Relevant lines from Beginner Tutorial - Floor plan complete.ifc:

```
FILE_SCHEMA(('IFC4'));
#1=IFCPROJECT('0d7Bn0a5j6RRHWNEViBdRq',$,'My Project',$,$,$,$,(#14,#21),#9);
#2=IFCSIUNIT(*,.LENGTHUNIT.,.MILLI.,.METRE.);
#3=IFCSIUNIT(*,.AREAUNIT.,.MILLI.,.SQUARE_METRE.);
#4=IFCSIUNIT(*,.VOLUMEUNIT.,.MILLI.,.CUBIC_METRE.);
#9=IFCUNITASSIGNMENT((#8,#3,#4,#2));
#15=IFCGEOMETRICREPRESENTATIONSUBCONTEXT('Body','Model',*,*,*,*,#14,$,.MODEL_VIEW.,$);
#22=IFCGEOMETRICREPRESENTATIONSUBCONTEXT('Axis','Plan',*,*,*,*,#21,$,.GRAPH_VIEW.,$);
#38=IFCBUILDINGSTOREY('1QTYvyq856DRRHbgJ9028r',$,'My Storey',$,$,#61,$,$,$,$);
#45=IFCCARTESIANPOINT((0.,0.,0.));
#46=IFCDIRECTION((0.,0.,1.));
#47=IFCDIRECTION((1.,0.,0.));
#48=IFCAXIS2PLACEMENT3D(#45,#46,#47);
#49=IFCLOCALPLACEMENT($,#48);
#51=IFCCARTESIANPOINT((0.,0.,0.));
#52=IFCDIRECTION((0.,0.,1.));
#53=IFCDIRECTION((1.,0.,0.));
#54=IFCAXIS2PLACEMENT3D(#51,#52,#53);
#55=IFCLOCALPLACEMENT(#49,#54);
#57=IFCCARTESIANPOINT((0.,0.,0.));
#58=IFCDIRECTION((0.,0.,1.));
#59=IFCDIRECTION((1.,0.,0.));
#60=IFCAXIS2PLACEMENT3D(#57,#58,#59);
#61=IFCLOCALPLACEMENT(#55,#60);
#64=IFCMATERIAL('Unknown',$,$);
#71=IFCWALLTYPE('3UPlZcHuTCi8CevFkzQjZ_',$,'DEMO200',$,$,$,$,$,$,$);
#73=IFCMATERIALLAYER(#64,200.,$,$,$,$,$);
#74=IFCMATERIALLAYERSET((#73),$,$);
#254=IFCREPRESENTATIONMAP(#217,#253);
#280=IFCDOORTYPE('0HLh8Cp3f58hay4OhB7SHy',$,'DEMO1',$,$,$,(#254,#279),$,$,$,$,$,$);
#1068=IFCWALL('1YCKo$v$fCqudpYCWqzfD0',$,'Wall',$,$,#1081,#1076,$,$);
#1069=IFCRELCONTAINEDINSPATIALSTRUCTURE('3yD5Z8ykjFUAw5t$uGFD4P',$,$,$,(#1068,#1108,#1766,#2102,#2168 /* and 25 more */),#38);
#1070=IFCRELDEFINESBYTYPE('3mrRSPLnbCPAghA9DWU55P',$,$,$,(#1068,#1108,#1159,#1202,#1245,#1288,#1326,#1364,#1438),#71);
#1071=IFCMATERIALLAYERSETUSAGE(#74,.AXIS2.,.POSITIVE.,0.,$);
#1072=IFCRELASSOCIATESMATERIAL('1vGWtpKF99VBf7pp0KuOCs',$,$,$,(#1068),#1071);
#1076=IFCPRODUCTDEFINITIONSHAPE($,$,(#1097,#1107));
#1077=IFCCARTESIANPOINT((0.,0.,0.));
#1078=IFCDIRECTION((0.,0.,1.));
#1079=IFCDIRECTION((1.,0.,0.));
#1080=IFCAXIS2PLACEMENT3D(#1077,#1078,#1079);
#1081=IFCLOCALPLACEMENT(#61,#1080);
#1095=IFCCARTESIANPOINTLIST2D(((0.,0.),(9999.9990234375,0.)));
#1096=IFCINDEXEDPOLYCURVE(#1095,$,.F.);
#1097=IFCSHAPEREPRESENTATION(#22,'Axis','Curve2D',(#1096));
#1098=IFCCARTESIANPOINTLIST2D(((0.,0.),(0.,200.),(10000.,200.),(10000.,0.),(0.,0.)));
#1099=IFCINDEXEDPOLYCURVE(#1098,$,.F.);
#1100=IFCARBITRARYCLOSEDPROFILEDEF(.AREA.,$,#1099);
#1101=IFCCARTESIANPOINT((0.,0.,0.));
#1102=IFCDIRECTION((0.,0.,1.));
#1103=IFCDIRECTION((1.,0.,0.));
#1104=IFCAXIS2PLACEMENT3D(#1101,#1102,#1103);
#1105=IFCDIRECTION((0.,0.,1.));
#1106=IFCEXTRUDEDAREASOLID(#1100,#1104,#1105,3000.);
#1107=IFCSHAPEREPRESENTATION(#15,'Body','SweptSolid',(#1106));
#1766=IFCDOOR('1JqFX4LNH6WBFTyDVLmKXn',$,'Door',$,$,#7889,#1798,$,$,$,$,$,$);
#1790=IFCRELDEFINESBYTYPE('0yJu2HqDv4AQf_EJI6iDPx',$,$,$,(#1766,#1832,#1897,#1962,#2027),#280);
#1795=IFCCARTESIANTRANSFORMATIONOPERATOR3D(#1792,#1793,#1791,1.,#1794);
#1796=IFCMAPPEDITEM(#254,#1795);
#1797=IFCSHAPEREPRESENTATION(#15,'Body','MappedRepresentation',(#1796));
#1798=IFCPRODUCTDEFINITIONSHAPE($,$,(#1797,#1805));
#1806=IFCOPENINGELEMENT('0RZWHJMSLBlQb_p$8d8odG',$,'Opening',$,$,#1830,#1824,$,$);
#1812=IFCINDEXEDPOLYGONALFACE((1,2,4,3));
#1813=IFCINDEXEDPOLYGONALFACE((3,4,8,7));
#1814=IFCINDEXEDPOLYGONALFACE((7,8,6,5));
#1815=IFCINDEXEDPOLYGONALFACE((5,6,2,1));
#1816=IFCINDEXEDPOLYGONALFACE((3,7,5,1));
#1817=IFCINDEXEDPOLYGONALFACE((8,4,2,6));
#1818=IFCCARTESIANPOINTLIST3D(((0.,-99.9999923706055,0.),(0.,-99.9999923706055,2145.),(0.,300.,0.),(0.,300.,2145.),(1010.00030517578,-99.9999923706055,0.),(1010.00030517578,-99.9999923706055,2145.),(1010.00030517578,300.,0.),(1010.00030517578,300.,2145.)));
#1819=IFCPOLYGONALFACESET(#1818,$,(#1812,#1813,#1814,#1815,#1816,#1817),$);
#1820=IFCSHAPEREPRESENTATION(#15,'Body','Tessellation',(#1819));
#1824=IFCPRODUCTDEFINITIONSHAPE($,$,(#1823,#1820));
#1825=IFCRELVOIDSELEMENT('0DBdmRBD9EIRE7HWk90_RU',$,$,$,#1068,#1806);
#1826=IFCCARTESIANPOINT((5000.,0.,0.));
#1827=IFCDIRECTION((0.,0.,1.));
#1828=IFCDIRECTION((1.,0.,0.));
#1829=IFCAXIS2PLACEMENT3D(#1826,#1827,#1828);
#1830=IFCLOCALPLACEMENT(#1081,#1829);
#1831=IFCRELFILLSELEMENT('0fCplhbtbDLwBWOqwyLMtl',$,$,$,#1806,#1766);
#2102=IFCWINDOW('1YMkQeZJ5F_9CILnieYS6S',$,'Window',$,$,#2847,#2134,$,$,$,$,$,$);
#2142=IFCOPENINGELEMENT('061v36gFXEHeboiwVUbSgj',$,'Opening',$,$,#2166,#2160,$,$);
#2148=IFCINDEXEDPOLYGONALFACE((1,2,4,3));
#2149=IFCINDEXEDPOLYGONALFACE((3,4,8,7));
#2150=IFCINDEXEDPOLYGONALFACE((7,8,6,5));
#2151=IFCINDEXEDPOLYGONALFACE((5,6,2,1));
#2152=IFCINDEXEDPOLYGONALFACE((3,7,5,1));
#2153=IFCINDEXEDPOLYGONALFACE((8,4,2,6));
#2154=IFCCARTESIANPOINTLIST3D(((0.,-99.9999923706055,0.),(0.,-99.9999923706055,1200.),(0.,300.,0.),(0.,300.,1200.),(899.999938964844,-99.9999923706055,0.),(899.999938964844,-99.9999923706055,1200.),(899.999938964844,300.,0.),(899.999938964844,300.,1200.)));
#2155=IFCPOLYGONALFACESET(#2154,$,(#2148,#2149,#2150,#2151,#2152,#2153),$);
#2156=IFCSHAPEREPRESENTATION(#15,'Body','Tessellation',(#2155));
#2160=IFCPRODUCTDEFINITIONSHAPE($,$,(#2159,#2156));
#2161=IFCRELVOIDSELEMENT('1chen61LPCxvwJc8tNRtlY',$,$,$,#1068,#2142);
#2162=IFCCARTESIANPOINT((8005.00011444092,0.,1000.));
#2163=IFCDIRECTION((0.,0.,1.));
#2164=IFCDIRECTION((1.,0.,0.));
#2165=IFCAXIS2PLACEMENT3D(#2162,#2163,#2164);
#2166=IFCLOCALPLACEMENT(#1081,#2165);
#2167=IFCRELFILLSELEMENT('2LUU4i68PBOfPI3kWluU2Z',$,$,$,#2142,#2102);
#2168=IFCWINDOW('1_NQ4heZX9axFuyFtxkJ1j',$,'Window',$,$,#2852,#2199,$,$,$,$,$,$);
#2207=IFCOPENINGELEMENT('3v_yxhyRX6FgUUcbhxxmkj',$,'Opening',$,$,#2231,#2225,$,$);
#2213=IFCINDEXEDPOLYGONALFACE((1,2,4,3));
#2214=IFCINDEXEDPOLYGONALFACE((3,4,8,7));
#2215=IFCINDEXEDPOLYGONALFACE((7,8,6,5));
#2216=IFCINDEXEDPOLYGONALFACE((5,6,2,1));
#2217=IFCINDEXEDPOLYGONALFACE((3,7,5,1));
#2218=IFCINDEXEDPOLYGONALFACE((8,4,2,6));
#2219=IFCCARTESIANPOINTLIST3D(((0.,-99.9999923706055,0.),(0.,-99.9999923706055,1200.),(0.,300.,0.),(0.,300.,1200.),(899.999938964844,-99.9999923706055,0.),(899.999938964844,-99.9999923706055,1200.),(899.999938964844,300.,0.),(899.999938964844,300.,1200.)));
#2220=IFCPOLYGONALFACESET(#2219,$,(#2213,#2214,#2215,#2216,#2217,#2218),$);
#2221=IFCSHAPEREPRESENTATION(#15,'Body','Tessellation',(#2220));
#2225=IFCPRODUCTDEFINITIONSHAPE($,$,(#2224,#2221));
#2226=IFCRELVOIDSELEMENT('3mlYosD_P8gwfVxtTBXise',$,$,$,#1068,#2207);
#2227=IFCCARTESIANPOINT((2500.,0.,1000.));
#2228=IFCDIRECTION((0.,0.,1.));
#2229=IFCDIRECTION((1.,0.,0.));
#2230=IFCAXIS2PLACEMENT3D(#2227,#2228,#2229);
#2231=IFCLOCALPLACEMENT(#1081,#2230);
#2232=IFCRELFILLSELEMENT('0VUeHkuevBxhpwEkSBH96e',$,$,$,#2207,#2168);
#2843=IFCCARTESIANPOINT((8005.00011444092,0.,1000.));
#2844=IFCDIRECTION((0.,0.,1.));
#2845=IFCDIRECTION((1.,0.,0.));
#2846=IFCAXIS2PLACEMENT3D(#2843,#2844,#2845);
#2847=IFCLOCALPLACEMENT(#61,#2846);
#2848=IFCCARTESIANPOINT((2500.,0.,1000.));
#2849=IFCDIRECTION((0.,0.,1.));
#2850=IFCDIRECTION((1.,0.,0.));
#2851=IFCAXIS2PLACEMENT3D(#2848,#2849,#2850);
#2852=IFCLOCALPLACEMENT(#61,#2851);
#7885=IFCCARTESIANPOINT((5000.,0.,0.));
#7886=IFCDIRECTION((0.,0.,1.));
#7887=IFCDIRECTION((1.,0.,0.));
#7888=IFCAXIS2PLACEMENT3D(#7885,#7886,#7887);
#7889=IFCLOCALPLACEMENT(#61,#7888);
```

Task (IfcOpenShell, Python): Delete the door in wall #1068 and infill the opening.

```python
import ifcopenshell
import ifcopenshell.api.feature
import ifcopenshell.api.root
import ifcopenshell.geom
import ifcopenshell.util.shape

model = ifcopenshell.open("Beginner Tutorial - Floor plan complete.ifc")
settings = ifcopenshell.geom.settings()


def volume(element):
    """Net volume in cubic metres, openings subtracted."""
    shape = ifcopenshell.geom.create_shape(settings, element)
    return ifcopenshell.util.shape.get_volume(shape.geometry)


door = model.by_id(1766)
opening = door.FillsVoids[0].RelatingOpeningElement
wall = opening.VoidsElements[0].RelatingBuildingElement
before = volume(wall)

ifcopenshell.api.root.remove_product(model, product=door)
ifcopenshell.api.feature.remove_feature(model, feature=opening)

after = volume(wall)

print(f"wall volume {before:.3f} -> {after:.3f} m3")

model.write("Beginner Tutorial - Floor plan complete_v2.ifc")
```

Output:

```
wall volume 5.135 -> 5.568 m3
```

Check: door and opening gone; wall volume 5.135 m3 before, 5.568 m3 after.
